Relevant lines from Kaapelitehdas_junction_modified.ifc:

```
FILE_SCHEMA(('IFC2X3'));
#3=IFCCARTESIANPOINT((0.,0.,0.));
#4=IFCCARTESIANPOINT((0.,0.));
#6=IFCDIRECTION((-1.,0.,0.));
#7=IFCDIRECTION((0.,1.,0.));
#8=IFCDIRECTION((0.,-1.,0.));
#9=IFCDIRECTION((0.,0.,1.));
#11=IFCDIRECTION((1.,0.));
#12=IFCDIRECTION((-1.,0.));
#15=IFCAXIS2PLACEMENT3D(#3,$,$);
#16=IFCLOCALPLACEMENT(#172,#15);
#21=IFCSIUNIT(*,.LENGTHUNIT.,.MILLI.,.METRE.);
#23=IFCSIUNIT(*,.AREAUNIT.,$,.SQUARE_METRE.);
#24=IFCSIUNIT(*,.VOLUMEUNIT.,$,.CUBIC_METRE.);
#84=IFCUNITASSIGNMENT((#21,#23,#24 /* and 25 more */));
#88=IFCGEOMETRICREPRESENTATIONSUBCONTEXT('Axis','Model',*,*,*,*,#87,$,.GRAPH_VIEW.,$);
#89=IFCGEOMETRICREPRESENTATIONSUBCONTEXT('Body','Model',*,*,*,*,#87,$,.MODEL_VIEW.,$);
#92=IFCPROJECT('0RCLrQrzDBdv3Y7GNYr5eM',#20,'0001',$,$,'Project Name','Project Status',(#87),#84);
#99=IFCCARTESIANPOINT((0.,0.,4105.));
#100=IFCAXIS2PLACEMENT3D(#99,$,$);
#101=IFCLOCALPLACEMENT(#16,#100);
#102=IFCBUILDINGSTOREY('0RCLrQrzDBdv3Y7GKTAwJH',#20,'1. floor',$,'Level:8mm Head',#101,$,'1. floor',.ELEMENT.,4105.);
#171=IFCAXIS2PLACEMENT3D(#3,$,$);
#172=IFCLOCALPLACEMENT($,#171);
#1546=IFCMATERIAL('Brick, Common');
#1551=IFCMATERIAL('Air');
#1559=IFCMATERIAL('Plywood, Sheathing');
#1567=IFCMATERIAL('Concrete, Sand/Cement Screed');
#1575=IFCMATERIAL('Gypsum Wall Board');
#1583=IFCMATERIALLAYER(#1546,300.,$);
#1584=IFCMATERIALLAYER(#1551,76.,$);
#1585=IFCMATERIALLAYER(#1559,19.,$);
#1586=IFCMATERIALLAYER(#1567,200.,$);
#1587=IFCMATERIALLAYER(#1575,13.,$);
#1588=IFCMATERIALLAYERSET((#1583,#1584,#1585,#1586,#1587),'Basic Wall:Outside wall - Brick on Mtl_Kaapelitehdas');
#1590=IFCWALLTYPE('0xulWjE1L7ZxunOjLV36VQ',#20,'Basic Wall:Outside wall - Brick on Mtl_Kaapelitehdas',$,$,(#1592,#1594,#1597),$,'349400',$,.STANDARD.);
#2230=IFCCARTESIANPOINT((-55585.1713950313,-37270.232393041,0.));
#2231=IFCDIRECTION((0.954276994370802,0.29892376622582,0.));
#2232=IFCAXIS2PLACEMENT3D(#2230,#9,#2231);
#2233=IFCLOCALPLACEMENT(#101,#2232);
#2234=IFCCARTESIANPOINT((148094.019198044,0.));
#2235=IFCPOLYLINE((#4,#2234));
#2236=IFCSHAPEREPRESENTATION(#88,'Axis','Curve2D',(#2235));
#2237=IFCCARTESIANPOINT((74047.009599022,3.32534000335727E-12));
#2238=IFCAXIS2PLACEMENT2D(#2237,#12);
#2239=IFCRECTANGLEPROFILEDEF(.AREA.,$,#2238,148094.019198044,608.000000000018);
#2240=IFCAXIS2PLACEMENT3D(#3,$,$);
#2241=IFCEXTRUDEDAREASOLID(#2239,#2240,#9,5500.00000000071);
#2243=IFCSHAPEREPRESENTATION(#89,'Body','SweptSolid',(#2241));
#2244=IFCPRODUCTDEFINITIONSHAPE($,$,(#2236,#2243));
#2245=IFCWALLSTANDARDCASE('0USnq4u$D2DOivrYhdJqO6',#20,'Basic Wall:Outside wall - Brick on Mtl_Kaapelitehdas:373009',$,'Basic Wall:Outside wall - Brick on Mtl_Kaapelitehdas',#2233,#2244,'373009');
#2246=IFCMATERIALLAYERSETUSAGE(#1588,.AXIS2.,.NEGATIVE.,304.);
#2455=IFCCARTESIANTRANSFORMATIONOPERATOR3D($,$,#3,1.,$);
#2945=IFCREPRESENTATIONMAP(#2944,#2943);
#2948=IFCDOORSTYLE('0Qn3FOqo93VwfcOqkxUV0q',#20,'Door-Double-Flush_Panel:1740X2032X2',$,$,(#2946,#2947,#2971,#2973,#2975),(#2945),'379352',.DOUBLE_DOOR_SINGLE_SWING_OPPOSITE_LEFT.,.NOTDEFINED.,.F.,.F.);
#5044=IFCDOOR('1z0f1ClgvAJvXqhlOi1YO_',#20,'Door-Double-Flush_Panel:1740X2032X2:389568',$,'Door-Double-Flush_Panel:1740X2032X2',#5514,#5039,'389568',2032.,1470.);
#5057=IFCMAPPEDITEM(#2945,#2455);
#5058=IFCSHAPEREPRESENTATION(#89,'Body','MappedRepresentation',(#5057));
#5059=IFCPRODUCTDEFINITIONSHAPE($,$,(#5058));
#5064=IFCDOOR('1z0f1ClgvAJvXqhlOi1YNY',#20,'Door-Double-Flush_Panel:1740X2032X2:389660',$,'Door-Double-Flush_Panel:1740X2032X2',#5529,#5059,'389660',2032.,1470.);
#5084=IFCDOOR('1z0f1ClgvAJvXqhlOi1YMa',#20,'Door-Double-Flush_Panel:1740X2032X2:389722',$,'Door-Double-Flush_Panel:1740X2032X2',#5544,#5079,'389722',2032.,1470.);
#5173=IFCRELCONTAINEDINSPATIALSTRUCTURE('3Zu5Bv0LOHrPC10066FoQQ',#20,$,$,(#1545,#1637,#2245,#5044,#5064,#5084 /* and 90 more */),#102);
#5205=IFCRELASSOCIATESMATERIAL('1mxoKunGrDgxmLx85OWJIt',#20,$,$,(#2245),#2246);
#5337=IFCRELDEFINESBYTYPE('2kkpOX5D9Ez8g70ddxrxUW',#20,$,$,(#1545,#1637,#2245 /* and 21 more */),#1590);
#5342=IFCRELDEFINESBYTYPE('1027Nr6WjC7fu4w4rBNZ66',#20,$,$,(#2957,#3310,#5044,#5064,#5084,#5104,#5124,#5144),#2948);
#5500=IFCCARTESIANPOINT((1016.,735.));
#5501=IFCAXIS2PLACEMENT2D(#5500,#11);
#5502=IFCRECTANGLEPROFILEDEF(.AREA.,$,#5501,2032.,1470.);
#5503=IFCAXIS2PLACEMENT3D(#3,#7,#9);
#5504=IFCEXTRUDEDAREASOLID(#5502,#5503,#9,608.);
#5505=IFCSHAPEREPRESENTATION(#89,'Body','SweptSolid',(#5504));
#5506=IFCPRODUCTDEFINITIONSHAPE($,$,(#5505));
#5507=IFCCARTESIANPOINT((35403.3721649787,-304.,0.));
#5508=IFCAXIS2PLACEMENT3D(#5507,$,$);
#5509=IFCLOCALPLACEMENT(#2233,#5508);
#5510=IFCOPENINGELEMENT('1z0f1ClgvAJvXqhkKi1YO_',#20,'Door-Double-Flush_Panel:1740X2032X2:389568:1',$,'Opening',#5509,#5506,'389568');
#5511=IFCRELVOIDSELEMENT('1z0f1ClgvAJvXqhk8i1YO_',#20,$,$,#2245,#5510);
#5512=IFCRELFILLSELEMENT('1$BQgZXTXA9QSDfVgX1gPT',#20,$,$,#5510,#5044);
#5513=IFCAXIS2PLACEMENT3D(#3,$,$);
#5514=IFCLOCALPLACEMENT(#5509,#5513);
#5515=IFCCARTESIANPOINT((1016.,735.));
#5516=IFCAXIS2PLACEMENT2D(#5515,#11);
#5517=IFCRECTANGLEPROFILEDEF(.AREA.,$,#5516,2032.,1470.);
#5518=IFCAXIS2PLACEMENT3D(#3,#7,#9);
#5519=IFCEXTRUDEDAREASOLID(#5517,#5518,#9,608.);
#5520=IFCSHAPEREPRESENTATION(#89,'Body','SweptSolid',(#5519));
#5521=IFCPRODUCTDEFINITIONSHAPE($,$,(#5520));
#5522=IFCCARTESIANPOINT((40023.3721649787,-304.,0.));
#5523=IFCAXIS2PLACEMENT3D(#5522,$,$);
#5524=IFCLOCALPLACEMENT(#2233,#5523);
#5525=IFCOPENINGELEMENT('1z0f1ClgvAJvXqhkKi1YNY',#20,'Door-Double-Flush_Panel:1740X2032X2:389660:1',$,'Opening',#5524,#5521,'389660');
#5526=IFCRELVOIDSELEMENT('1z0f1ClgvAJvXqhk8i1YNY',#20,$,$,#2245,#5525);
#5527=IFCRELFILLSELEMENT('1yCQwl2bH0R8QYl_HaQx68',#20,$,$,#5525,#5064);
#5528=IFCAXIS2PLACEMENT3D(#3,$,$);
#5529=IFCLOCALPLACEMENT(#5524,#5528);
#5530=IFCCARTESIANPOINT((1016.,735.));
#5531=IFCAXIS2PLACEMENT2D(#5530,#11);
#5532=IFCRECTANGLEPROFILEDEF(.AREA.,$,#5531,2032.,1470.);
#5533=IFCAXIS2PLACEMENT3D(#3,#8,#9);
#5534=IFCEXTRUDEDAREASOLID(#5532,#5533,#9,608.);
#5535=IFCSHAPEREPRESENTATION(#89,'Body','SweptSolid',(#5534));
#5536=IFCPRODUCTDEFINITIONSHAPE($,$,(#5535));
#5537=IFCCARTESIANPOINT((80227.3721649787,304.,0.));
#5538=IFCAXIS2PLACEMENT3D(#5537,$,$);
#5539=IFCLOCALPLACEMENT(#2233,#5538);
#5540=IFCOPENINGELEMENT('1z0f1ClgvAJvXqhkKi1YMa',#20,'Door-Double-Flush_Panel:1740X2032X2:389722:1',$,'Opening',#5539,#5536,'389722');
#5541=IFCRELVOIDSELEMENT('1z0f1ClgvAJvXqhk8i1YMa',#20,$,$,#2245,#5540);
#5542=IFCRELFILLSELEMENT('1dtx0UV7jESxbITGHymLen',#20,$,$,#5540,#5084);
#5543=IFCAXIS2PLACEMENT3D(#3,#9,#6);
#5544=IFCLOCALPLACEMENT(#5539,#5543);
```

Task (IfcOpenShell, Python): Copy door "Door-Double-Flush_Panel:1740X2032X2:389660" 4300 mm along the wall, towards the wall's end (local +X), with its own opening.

```python
import ifcopenshell
import ifcopenshell.api.feature
import ifcopenshell.api.geometry
import ifcopenshell.api.root
import ifcopenshell.geom
import ifcopenshell.util.element
import ifcopenshell.util.placement
import ifcopenshell.util.shape

model = ifcopenshell.open("Kaapelitehdas_junction_modified.ifc")
settings = ifcopenshell.geom.settings()


def volume(element):
    """Net volume in cubic metres, openings subtracted."""
    shape = ifcopenshell.geom.create_shape(settings, element)
    return ifcopenshell.util.shape.get_volume(shape.geometry)


def reuse_history(source, copy):
    """copy_class also copies each property set's owner history, people and application; keep the originals."""
    for rel in copy.IsDefinedBy:
        if rel.is_a("IfcRelDefinesByProperties") and (history := rel.RelatingPropertyDefinition.OwnerHistory):
            rel.RelatingPropertyDefinition.OwnerHistory = source.OwnerHistory
            ifcopenshell.util.element.remove_deep2(model, history)


door = model.by_guid("1z0f1ClgvAJvXqhlOi1YNY")
opening = door.FillsVoids[0].RelatingOpeningElement
wall = opening.VoidsElements[0].RelatingBuildingElement
before = volume(wall)
shift = ifcopenshell.util.placement.get_local_placement(wall.ObjectPlacement)[:3, 0] * 4300.0

# copy_class copies the void relationship, type, container and properties, but no geometry.
new_opening = ifcopenshell.api.root.copy_class(model, product=opening)
new_opening.Representation = ifcopenshell.util.element.copy_deep(
    model, opening.Representation, exclude=["IfcGeometricRepresentationContext", "IfcRepresentationMap"]
)
new_opening.Name = "Door-Double-Flush_Panel:1740X2032X2"
new_opening.Tag = None
new_door = ifcopenshell.api.root.copy_class(model, product=door)
new_door.Representation = ifcopenshell.util.element.copy_deep(
    model, door.Representation, exclude=["IfcGeometricRepresentationContext", "IfcRepresentationMap"]
)
new_door.Name = "Door-Double-Flush_Panel:1740X2032X2"
new_door.Tag = None
reuse_history(door, new_door)
fills = ifcopenshell.api.feature.add_filling(model, opening=new_opening, element=new_door)
fills.OwnerHistory = new_door.OwnerHistory  # required in IFC2X3

for old, new in ((opening, new_opening), (door, new_door)):
    matrix = ifcopenshell.util.placement.get_local_placement(old.ObjectPlacement)
    matrix[:3, 3] += shift
    ifcopenshell.api.geometry.edit_object_placement(model, product=new, matrix=matrix, is_si=False)

after = volume(wall)

print(f"wall volume {before:.3f} -> {after:.3f} m3")

model.write("Kaapelitehdas_junction_modified_updated.ifc")
```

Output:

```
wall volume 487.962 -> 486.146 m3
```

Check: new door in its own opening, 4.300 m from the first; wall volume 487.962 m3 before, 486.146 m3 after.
